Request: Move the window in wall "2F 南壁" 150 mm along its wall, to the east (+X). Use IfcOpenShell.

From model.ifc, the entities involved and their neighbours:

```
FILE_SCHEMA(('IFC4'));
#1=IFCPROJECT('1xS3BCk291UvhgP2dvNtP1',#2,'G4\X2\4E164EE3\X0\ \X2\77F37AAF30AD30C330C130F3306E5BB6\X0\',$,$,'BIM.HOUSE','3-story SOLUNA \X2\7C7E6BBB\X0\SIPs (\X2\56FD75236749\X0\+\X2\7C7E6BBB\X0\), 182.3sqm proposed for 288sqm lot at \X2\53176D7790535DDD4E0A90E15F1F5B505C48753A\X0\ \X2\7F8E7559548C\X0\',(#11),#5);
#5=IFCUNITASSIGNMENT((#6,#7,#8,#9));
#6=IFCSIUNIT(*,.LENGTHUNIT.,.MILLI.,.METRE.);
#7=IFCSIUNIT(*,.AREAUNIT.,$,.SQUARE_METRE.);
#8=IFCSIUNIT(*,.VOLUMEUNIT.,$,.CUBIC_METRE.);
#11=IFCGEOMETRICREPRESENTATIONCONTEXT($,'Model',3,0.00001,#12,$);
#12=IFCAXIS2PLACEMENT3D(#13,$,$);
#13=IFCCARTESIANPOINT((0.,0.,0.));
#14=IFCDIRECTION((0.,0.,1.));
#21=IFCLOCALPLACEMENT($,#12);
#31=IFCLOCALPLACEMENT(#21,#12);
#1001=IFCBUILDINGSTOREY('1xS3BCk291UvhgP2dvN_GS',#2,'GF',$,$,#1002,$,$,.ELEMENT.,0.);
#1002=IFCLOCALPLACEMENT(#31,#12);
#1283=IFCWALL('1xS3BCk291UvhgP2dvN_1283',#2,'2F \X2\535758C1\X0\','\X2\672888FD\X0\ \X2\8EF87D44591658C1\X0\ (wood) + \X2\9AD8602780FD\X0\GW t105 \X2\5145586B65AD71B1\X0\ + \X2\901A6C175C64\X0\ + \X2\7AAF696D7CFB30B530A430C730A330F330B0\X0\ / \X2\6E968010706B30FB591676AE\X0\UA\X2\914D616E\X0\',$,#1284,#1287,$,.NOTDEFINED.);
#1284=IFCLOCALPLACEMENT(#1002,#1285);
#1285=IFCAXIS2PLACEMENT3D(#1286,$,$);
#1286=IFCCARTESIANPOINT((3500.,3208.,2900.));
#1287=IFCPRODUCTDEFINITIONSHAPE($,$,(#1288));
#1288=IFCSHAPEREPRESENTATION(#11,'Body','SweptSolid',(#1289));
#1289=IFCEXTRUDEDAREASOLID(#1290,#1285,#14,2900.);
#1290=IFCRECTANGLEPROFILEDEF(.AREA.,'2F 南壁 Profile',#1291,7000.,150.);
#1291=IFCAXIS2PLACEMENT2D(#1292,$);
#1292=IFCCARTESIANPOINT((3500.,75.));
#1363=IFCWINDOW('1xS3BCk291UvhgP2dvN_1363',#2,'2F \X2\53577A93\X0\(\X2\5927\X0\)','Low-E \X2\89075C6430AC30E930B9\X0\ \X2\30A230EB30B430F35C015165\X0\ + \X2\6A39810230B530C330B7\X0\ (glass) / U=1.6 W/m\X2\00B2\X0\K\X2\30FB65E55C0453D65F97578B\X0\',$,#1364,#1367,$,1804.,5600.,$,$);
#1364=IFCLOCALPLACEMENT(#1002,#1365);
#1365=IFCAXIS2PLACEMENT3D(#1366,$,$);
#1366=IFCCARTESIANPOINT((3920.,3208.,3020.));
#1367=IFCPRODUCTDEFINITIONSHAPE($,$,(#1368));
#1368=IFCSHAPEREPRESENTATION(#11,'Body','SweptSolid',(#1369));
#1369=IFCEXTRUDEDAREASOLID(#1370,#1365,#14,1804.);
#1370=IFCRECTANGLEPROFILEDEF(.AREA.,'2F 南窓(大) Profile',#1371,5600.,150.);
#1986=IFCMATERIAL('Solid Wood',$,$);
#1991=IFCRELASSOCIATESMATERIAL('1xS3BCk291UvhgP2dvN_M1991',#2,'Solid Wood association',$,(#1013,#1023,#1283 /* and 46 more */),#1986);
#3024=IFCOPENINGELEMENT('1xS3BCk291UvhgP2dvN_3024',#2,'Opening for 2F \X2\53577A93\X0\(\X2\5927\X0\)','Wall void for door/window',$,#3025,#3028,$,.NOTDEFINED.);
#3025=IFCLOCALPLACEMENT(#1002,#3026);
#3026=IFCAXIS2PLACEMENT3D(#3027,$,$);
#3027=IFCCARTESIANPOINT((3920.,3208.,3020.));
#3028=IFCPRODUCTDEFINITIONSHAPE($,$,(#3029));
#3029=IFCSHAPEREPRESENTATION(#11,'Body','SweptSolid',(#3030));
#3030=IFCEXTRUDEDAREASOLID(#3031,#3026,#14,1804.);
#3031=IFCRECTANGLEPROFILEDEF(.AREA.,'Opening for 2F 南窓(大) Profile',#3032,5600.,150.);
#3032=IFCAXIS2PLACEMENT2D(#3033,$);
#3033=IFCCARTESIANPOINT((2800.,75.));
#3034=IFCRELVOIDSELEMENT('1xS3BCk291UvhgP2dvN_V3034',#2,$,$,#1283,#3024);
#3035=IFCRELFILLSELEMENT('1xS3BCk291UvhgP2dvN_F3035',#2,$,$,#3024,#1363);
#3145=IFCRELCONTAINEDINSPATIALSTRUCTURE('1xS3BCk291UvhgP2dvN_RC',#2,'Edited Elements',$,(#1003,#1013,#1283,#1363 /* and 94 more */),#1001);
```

```python
import ifcopenshell
import ifcopenshell.api.geometry
import ifcopenshell.util.placement

model = ifcopenshell.open("model.ifc")

window = model.by_guid("1xS3BCk291UvhgP2dvN_1363")
opening = window.FillsVoids[0].RelatingOpeningElement
wall = opening.VoidsElements[0].RelatingBuildingElement

wall_matrix = ifcopenshell.util.placement.get_local_placement(wall.ObjectPlacement)
shift = wall_matrix[:3, 0] * 150.0
before = ifcopenshell.util.placement.get_local_placement(window.ObjectPlacement)[:3, 3].copy()

# The window is not placed relative to its opening, so move both.
for product in (opening, window):
    matrix = ifcopenshell.util.placement.get_local_placement(product.ObjectPlacement)
    matrix[:3, 3] += shift
    ifcopenshell.api.geometry.edit_object_placement(model, product=product, matrix=matrix, is_si=False)

after = ifcopenshell.util.placement.get_local_placement(window.ObjectPlacement)[:3, 3]
print("window moved by", (after - before).round(3) + 0.0)

model.write("model_rev.ifc")
```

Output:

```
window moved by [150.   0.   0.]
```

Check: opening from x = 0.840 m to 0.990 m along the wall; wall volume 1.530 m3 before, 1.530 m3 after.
